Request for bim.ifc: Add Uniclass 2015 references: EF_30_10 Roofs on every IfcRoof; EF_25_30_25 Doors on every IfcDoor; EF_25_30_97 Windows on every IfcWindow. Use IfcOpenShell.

First a look at what the model holds.

```python
import ifcopenshell

model = ifcopenshell.open("bim.ifc")
print(model.schema)
print("classifications:", [c.Name for c in model.by_type("IfcClassification")])
for ifc_class in ("IfcDoor", "IfcRoof", "IfcStair", "IfcWall", "IfcWindow"):
    print(ifc_class, len(model.by_type(ifc_class)))
```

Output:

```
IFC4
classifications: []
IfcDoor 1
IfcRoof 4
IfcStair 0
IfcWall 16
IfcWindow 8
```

```python
import ifcopenshell
import ifcopenshell.api.classification

model = ifcopenshell.open("bim.ifc")

system = ifcopenshell.api.classification.add_classification(model, classification="Uniclass 2015")

codes = {
    "IfcRoof": ("EF_30_10", "Roofs"),
    "IfcDoor": ("EF_25_30_25", "Doors"),
    "IfcWindow": ("EF_25_30_97", "Windows"),
}
for ifc_class, (code, name) in codes.items():
    products = model.by_type(ifc_class)
    ifcopenshell.api.classification.add_reference(
        model, products=products, classification=system, identification=code, name=name
    )
    print(code, len(products))

model.write("bim_updated.ifc")
```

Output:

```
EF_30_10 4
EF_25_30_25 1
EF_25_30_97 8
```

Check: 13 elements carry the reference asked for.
